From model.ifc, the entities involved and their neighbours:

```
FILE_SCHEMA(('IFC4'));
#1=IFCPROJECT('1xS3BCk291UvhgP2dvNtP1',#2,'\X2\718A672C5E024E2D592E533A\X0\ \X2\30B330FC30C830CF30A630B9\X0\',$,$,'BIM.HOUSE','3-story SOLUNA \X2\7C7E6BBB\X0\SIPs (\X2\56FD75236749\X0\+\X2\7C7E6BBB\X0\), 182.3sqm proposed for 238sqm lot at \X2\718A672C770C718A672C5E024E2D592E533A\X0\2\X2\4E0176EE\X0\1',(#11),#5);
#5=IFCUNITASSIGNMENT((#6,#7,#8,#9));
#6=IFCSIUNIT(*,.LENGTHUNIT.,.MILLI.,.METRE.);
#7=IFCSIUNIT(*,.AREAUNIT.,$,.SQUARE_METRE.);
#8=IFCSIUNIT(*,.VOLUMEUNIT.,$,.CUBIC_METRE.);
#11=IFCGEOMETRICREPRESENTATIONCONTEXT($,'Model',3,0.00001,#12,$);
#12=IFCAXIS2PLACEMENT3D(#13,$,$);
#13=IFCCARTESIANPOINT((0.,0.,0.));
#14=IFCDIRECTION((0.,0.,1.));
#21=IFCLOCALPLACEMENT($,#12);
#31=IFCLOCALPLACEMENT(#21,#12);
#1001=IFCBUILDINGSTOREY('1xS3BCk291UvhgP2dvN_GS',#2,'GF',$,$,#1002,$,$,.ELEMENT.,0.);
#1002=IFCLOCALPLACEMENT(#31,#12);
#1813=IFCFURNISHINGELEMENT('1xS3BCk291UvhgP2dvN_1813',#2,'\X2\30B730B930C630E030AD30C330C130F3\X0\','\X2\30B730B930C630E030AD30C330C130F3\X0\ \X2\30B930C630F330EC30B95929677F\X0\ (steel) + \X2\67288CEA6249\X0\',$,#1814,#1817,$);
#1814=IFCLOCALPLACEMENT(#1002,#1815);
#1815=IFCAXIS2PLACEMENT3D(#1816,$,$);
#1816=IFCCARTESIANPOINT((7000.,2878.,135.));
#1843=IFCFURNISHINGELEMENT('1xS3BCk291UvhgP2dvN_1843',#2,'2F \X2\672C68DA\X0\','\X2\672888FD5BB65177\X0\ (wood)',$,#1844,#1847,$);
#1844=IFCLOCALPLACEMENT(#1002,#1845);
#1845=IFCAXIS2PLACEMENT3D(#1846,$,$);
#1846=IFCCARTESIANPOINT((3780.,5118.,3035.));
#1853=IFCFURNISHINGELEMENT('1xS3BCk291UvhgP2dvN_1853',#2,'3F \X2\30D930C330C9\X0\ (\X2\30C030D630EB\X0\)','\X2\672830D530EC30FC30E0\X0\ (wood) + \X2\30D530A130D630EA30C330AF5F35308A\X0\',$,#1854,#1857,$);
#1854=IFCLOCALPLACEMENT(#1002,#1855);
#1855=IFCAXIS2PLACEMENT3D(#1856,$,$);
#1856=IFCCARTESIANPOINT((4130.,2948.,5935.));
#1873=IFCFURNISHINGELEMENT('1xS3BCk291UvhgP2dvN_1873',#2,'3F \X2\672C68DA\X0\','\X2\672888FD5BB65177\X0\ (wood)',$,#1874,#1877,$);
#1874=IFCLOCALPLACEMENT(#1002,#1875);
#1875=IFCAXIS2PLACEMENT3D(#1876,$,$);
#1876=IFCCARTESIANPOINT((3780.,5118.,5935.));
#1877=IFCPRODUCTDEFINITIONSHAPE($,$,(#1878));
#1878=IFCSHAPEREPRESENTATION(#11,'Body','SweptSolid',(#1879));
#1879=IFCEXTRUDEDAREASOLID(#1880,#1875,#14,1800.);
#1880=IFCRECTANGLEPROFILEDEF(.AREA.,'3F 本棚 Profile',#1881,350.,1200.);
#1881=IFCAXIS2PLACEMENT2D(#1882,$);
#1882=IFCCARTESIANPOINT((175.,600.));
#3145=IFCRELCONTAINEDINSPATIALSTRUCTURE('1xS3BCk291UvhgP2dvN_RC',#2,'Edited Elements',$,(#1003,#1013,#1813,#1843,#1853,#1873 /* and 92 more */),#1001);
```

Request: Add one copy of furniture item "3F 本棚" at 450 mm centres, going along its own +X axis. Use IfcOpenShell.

```python
import ifcopenshell
import ifcopenshell.api.geometry
import ifcopenshell.api.root
import ifcopenshell.util.element
import ifcopenshell.util.placement
import ifcopenshell.util.unit

model = ifcopenshell.open("model.ifc")
unit_scale = ifcopenshell.util.unit.calculate_unit_scale(model)


def reuse_history(source, copy):
    """copy_class also copies each property set's owner history, people and application; keep the originals."""
    for rel in copy.IsDefinedBy:
        if rel.is_a("IfcRelDefinesByProperties") and (history := rel.RelatingPropertyDefinition.OwnerHistory):
            rel.RelatingPropertyDefinition.OwnerHistory = source.OwnerHistory
            ifcopenshell.util.element.remove_deep2(model, history)


source = model.by_guid("1xS3BCk291UvhgP2dvN_1873")
base = ifcopenshell.util.placement.get_local_placement(source.ObjectPlacement)
step = base[:3, 0] * 0.45 / unit_scale

for i in range(1, 2):
    copy = ifcopenshell.api.root.copy_class(model, product=source)
    copy.Representation = ifcopenshell.util.element.copy_deep(
        model, source.Representation, exclude=["IfcGeometricRepresentationContext", "IfcRepresentationMap"]
    )
    reuse_history(source, copy)
    matrix = base.copy()
    matrix[:3, 3] += i * step
    print("added at", matrix[:3, 3].round(3) + 0.0)
    ifcopenshell.api.geometry.edit_object_placement(model, product=copy, matrix=matrix, is_si=False)

model.write("model-out.ifc")
```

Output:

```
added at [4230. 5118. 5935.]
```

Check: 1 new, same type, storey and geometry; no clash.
